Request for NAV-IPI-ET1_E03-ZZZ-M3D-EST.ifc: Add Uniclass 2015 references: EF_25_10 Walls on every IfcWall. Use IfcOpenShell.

First a look at what the model holds.

```python
import ifcopenshell

model = ifcopenshell.open("NAV-IPI-ET1_E03-ZZZ-M3D-EST.ifc")
print(model.schema)
print("classifications:", [c.Name for c in model.by_type("IfcClassification")])
for ifc_class in ("IfcDoor", "IfcRoof", "IfcStair", "IfcWall", "IfcWindow"):
    print(ifc_class, len(model.by_type(ifc_class)))
```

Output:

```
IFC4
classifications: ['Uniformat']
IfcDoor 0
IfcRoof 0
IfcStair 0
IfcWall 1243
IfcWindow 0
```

```python
import ifcopenshell
import ifcopenshell.api.classification

model = ifcopenshell.open("NAV-IPI-ET1_E03-ZZZ-M3D-EST.ifc")

system = ifcopenshell.api.classification.add_classification(model, classification="Uniclass 2015")

codes = {
    "IfcWall": ("EF_25_10", "Walls"),
}
for ifc_class, (code, name) in codes.items():
    products = model.by_type(ifc_class)
    ifcopenshell.api.classification.add_reference(
        model, products=products, classification=system, identification=code, name=name
    )
    print(code, len(products))

model.write("NAV-IPI-ET1_E03-ZZZ-M3D-EST_rev.ifc")
```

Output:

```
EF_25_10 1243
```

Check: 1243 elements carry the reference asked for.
